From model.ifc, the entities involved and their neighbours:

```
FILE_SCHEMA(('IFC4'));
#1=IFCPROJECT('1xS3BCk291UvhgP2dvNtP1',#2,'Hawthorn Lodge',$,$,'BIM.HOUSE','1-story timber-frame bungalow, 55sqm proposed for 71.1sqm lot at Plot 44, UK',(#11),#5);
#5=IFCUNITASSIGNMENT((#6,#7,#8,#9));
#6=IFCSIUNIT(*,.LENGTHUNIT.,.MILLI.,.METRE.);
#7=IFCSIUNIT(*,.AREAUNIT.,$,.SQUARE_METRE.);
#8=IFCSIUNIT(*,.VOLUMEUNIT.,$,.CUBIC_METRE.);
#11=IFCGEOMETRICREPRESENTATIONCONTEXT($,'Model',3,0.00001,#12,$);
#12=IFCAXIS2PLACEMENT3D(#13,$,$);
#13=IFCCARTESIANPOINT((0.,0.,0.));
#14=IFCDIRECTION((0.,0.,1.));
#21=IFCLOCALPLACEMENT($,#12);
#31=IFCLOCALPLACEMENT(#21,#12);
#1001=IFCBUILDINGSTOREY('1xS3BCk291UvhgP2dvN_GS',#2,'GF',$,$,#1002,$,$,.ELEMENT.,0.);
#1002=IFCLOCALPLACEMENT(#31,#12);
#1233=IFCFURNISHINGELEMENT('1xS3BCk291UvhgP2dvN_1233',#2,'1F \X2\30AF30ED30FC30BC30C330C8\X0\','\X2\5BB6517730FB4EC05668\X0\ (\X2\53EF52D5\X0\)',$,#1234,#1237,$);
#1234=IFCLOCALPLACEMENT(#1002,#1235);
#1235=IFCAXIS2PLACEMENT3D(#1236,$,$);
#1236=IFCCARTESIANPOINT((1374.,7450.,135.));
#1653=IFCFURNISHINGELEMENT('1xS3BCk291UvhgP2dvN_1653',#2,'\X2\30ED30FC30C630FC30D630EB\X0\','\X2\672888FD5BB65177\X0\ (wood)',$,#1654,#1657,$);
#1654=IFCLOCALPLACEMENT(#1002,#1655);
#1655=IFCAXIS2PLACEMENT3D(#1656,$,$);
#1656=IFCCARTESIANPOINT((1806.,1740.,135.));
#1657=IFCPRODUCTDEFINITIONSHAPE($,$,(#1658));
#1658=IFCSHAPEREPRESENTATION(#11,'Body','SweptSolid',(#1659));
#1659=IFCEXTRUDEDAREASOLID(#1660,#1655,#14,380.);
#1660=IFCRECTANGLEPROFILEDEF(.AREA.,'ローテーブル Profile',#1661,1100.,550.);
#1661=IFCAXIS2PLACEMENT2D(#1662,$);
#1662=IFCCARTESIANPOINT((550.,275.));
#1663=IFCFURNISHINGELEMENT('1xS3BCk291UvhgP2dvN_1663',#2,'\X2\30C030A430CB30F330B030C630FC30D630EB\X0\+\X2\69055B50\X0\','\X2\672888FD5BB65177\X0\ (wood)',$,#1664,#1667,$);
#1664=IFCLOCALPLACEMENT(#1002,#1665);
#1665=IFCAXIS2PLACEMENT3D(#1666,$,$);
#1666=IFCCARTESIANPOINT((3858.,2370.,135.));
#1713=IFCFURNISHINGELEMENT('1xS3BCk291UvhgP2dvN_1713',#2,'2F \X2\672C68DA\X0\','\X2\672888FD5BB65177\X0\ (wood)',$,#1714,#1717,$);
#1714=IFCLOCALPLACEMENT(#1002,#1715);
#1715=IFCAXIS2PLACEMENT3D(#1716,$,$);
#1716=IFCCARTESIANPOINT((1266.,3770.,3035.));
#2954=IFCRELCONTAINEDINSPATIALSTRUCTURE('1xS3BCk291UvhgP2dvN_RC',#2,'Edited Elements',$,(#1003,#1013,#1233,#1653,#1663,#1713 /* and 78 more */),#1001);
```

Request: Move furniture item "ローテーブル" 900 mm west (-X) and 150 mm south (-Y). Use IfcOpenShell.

```python
import ifcopenshell
import ifcopenshell.api.geometry
import ifcopenshell.util.placement
import ifcopenshell.util.unit

model = ifcopenshell.open("model.ifc")
unit_scale = ifcopenshell.util.unit.calculate_unit_scale(model)

item = model.by_id(1653)
matrix = ifcopenshell.util.placement.get_local_placement(item.ObjectPlacement)
matrix[0, 3] -= 0.9 / unit_scale
matrix[1, 3] -= 0.15 / unit_scale
ifcopenshell.api.geometry.edit_object_placement(model, product=item, matrix=matrix, is_si=False)

print(ifcopenshell.util.placement.get_local_placement(item.ObjectPlacement).round(3) + 0.0)

model.write("model_updated.ifc")
```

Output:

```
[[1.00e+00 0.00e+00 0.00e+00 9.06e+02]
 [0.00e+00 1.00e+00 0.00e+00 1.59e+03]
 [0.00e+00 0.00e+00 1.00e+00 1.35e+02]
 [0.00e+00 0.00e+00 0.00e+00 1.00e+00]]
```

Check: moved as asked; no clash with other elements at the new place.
